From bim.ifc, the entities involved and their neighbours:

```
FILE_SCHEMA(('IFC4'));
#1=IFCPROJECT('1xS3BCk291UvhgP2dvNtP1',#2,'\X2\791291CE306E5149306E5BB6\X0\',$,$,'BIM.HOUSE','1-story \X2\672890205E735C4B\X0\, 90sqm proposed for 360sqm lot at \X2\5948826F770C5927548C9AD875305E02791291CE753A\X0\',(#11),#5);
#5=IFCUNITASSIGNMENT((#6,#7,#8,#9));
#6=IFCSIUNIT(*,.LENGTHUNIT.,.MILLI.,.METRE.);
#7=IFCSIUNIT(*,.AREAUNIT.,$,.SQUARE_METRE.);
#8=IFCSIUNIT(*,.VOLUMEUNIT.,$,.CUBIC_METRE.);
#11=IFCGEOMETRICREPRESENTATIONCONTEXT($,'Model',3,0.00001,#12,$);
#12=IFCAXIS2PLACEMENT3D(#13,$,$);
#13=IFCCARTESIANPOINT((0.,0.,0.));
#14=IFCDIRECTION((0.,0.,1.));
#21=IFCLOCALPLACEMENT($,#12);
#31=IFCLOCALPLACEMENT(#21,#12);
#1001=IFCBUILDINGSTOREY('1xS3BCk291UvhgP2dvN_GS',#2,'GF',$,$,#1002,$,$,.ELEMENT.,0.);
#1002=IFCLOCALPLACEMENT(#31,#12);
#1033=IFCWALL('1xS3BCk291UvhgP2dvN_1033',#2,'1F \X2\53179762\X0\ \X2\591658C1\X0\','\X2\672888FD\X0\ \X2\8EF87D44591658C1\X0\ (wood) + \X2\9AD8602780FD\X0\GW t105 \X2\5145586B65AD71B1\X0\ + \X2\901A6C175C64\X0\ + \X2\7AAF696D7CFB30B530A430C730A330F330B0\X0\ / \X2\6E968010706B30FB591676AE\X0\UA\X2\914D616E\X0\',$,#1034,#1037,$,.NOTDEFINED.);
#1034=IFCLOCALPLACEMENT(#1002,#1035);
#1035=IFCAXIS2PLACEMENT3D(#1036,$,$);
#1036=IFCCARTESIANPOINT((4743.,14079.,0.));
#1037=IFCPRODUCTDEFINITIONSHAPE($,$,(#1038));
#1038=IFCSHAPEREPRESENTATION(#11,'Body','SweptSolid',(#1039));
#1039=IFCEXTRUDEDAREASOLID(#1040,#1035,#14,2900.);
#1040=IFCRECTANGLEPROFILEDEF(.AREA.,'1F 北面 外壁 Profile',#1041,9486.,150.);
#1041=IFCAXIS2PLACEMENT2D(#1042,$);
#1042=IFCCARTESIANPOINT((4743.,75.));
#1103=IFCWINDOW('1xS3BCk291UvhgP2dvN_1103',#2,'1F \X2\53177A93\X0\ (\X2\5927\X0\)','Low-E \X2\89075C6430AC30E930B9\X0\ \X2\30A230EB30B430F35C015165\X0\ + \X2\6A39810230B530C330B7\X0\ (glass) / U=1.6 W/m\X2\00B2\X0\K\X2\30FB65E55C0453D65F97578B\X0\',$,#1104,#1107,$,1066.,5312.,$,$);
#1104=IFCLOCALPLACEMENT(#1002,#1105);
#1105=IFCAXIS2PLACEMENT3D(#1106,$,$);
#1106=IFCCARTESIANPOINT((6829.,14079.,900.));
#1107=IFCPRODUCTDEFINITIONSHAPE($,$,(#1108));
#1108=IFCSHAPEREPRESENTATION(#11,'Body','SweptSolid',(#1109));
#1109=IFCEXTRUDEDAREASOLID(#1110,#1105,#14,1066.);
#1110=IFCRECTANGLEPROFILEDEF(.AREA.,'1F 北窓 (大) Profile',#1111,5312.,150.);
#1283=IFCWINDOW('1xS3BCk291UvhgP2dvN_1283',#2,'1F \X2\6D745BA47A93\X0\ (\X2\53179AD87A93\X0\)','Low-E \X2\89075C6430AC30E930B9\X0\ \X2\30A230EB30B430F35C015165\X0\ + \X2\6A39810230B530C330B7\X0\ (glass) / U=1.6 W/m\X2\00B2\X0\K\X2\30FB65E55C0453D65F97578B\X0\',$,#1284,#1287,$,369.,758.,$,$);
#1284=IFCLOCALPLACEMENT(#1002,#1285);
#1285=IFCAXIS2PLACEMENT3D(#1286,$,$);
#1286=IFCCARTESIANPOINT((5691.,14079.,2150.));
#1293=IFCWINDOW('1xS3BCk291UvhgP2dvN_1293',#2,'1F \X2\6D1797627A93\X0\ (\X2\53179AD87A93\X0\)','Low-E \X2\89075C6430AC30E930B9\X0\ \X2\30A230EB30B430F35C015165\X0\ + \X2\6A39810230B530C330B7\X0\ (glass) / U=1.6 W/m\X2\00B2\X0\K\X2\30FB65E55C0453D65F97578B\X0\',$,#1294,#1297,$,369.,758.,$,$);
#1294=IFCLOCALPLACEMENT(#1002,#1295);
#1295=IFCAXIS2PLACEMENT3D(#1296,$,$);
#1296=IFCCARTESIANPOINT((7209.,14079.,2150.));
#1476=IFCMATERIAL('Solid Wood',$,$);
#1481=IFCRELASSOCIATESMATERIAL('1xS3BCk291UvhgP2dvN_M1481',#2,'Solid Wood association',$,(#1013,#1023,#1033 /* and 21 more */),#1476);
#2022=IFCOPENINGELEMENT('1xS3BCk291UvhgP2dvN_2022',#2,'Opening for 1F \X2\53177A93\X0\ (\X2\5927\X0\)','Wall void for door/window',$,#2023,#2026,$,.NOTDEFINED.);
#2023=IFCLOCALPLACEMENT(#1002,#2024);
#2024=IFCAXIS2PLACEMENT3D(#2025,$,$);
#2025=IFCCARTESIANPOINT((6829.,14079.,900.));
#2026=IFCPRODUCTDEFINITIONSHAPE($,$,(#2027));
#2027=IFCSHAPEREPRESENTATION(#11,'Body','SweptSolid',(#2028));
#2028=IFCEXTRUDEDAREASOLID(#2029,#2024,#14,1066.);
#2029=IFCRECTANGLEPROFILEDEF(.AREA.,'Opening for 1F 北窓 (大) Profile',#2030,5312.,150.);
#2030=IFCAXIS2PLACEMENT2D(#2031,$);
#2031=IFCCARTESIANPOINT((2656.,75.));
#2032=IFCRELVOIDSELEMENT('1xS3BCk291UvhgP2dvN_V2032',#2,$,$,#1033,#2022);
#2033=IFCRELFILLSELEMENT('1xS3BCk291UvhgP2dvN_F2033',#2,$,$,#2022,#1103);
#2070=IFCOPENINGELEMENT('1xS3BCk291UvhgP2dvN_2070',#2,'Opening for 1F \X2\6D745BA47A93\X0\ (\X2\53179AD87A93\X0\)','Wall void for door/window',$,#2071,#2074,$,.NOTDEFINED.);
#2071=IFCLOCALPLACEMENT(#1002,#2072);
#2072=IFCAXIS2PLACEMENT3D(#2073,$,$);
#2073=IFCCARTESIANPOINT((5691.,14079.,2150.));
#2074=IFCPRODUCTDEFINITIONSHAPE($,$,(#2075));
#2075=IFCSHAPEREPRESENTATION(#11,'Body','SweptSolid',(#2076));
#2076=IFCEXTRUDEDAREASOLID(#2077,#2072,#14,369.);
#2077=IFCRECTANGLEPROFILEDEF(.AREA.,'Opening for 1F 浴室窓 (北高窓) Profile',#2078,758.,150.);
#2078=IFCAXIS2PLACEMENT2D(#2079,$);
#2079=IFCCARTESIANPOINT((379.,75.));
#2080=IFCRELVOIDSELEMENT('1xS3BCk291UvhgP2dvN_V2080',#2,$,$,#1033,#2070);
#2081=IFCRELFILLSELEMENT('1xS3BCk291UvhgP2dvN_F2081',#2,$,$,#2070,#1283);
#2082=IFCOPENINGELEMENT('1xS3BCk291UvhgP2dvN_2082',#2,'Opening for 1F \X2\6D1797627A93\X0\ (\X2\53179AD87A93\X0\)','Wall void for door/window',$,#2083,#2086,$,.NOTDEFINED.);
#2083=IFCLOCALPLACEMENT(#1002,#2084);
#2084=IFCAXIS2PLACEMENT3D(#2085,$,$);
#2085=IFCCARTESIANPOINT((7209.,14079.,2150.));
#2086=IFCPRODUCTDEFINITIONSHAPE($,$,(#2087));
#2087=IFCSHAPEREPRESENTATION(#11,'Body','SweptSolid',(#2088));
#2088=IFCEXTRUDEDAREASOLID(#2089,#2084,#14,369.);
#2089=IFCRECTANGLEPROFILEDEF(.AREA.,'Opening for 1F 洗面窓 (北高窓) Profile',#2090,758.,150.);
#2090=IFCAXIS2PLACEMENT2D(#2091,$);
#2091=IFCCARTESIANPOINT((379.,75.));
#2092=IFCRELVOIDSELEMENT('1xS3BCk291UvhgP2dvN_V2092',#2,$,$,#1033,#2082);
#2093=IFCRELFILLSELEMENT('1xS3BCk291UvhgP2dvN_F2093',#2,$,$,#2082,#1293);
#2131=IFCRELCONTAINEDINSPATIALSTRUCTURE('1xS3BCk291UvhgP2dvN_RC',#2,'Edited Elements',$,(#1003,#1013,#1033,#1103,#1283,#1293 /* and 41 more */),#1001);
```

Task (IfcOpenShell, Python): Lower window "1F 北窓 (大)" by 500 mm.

```python
import numpy as np
import ifcopenshell
import ifcopenshell.api.geometry
import ifcopenshell.util.placement
import ifcopenshell.util.unit

model = ifcopenshell.open("bim.ifc")
unit_scale = ifcopenshell.util.unit.calculate_unit_scale(model)

window = model.by_guid("1xS3BCk291UvhgP2dvN_1103")
opening = window.FillsVoids[0].RelatingOpeningElement
dz = -500.0

shift = np.array([0.0, 0.0, dz])
# The window is not placed relative to its opening, so move both.
for product in (opening, window):
    matrix = ifcopenshell.util.placement.get_local_placement(product.ObjectPlacement)
    matrix[:3, 3] += shift
    ifcopenshell.api.geometry.edit_object_placement(model, product=product, matrix=matrix, is_si=False)

print(f"moved by {dz * unit_scale:+.3f} m")

model.write("bim-out.ifc")
```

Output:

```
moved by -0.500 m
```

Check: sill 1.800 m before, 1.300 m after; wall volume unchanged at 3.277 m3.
